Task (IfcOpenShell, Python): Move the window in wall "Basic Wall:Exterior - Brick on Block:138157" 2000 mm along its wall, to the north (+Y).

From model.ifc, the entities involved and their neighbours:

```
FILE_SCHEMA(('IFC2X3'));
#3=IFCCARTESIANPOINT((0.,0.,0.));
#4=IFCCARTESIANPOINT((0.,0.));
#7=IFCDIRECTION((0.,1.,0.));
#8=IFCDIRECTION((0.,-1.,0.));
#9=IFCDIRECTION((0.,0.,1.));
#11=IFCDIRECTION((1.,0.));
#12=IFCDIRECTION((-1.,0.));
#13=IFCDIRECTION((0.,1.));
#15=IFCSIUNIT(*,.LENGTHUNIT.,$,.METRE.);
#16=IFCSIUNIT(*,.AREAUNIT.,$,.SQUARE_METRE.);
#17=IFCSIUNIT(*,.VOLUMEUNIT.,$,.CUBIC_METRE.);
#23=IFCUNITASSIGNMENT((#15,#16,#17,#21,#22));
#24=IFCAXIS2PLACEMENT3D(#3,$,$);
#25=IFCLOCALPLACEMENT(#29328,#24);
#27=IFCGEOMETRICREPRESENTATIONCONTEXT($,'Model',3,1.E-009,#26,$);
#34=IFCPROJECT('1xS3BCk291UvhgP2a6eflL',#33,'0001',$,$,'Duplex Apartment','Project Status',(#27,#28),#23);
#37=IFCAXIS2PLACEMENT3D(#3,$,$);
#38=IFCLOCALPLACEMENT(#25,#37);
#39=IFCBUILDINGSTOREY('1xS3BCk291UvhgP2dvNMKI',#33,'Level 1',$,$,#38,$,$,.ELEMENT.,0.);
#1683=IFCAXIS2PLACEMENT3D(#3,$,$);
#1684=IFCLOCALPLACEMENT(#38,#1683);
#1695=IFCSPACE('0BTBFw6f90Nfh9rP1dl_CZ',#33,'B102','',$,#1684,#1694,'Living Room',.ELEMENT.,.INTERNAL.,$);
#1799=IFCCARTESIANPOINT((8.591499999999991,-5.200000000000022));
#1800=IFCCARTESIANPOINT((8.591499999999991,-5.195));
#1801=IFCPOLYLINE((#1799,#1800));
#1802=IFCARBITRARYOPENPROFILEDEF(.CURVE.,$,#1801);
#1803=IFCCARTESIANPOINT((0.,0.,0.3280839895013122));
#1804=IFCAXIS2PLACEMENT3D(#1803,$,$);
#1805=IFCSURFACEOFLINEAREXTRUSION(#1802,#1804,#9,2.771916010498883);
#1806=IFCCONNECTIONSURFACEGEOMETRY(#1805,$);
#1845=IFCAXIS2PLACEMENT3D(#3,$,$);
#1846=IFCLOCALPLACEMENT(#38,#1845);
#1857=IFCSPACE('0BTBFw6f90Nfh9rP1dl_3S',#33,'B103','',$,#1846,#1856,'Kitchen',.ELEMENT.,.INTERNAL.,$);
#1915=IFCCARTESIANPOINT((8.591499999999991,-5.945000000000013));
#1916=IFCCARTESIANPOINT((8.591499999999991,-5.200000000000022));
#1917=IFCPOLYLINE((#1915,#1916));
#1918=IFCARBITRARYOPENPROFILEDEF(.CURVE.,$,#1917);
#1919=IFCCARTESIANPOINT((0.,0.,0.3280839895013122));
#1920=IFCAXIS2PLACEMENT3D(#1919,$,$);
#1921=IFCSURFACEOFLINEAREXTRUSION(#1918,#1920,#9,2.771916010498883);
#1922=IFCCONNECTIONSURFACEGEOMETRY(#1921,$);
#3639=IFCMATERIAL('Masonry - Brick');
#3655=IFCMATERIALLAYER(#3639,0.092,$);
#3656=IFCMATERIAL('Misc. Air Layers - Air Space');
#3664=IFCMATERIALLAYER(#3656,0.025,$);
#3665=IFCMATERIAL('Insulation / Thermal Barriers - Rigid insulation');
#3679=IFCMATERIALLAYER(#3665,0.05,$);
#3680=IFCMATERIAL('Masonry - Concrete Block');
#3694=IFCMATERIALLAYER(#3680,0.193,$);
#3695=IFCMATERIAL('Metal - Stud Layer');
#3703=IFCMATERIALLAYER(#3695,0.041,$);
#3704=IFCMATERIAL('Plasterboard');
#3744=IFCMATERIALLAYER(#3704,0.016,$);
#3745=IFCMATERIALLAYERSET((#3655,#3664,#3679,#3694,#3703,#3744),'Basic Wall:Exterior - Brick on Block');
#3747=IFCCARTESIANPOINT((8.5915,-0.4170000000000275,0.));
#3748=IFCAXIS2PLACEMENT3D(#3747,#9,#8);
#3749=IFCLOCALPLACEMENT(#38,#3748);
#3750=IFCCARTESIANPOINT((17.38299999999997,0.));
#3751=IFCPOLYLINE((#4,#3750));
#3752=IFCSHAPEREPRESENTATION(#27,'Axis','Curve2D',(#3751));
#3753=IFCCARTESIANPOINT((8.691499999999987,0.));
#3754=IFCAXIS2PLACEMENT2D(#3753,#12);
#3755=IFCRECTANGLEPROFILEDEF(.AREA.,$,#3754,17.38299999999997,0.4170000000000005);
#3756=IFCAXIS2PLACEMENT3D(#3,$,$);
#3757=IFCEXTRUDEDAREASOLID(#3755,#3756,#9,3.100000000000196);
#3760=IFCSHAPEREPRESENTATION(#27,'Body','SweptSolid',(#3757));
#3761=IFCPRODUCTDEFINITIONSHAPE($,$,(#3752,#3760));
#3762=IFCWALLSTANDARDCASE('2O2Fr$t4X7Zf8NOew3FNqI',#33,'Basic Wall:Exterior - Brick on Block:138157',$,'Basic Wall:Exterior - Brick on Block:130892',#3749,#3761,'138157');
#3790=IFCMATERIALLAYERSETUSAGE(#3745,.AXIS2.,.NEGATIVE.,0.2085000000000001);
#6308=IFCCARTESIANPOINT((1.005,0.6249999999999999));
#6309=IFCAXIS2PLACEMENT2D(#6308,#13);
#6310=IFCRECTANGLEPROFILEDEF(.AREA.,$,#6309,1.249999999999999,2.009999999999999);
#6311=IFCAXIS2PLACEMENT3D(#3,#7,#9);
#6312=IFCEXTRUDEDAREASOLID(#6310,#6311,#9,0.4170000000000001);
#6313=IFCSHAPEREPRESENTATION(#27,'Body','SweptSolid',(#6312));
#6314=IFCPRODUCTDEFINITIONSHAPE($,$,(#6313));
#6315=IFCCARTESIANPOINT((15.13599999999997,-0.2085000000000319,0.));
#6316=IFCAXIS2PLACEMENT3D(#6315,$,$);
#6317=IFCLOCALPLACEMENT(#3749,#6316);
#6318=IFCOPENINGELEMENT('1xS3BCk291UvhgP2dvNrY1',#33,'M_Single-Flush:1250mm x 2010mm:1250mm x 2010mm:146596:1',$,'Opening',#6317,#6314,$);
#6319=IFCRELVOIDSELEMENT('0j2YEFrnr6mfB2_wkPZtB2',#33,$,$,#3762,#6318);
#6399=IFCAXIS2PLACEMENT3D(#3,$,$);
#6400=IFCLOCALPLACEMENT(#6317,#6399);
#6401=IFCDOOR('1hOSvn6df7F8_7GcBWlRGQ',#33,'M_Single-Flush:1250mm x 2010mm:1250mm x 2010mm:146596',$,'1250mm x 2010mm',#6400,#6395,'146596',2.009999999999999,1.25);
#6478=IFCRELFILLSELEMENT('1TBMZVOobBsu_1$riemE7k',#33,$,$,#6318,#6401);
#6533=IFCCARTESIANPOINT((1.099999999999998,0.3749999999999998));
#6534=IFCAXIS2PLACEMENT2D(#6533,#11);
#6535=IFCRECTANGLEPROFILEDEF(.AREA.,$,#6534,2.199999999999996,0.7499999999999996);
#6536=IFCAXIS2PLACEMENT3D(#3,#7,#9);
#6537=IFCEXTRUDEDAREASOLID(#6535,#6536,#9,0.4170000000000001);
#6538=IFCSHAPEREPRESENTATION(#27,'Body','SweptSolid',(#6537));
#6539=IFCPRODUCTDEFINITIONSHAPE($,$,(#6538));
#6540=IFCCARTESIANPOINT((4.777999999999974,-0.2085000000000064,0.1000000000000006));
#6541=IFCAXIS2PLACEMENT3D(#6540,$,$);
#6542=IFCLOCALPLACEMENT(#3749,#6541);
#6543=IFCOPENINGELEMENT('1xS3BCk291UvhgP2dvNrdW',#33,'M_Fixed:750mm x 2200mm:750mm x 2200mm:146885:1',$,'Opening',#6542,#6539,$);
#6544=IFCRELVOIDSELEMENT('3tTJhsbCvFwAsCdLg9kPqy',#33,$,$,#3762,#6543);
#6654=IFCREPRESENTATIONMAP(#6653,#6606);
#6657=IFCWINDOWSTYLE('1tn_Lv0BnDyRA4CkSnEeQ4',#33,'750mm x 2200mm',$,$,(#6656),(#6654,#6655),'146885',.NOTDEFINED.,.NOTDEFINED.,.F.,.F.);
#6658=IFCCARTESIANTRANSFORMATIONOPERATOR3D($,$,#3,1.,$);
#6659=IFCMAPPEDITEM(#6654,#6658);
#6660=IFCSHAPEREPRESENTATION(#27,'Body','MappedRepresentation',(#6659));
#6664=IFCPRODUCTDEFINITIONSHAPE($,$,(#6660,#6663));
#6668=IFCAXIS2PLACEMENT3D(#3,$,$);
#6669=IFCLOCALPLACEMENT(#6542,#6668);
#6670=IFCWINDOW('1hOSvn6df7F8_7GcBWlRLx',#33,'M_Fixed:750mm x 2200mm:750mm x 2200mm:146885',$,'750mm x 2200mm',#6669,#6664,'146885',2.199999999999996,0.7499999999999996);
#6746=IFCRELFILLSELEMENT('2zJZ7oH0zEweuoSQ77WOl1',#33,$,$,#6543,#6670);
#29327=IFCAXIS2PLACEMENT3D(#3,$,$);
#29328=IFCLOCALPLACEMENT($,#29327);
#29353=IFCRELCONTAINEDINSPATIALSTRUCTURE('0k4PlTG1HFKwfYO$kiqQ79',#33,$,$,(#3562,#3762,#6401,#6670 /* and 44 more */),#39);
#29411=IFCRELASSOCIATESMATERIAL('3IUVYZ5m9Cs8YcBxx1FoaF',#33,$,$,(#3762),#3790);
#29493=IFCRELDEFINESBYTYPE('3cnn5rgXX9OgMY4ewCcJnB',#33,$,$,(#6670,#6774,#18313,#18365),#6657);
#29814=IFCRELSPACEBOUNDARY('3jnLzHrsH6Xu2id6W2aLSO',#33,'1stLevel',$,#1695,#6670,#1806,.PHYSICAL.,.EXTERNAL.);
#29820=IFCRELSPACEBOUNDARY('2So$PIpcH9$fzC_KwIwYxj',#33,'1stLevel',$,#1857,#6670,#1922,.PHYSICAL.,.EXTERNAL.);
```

```python
import numpy as np
import ifcopenshell
import ifcopenshell.api.geometry
import ifcopenshell.util.placement

model = ifcopenshell.open("model.ifc")

window = model.by_guid("1hOSvn6df7F8_7GcBWlRLx")
opening = window.FillsVoids[0].RelatingOpeningElement
wall = opening.VoidsElements[0].RelatingBuildingElement

wall_matrix = ifcopenshell.util.placement.get_local_placement(wall.ObjectPlacement)
shift = wall_matrix[:3, 0] * -2.0
before = ifcopenshell.util.placement.get_local_placement(window.ObjectPlacement)[:3, 3].copy()

# The window is placed relative to its opening, so it follows when the opening moves.
matrix = ifcopenshell.util.placement.get_local_placement(opening.ObjectPlacement)
matrix[:3, 3] += shift
ifcopenshell.api.geometry.edit_object_placement(
    model, product=opening, matrix=matrix, is_si=False, should_transform_children=True
)

# Space boundary surfaces are stored in each space's coordinates; move them too.
for rel in window.ProvidesBoundaries:
    if not rel.ConnectionGeometry:
        continue
    surface = rel.ConnectionGeometry.SurfaceOnRelatingElement
    space_matrix = ifcopenshell.util.placement.get_local_placement(rel.RelatingSpace.ObjectPlacement)
    point = np.array(surface.Position.Location.Coordinates) + space_matrix[:3, :3].T @ shift
    surface.Position = model.createIfcAxis2Placement3D(
        model.createIfcCartesianPoint(point.tolist()), surface.Position.Axis, surface.Position.RefDirection
    )

after = ifcopenshell.util.placement.get_local_placement(window.ObjectPlacement)[:3, 3]
print("window moved by", (after - before).round(3) + 0.0)

model.write("model_updated.ifc")
```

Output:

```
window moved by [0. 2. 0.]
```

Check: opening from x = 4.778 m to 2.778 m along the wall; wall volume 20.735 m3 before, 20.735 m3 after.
